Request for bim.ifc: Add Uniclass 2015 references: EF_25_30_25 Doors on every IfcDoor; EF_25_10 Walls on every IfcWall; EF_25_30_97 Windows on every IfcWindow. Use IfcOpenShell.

First a look at what the model holds.

```python
import ifcopenshell

model = ifcopenshell.open("bim.ifc")
print(model.schema)
print("classifications:", [c.Name for c in model.by_type("IfcClassification")])
for ifc_class in ("IfcDoor", "IfcRoof", "IfcStair", "IfcWall", "IfcWindow"):
    print(ifc_class, len(model.by_type(ifc_class)))
```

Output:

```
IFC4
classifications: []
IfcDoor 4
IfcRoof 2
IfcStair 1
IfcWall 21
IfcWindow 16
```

```python
import ifcopenshell
import ifcopenshell.api.classification

model = ifcopenshell.open("bim.ifc")

system = ifcopenshell.api.classification.add_classification(model, classification="Uniclass 2015")

codes = {
    "IfcDoor": ("EF_25_30_25", "Doors"),
    "IfcWall": ("EF_25_10", "Walls"),
    "IfcWindow": ("EF_25_30_97", "Windows"),
}
for ifc_class, (code, name) in codes.items():
    products = model.by_type(ifc_class)
    ifcopenshell.api.classification.add_reference(
        model, products=products, classification=system, identification=code, name=name
    )
    print(code, len(products))

model.write("bim_v2.ifc")
```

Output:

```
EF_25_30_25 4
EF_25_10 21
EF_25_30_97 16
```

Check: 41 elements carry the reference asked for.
